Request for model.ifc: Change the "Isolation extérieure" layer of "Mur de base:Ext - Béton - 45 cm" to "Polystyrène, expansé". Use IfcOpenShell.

First a look at what the model holds.

```python
import ifcopenshell
import ifcopenshell.util.element

model = ifcopenshell.open("model.ifc")
print(model.schema)
for layer_set in model.by_type("IfcMaterialLayerSet"):
    if layer_set.LayerSetName == "Mur de base:Ext - Béton - 45 cm":
        for layer in layer_set.MaterialLayers:
            print(layer.id(), layer.Material and layer.Material.Name, layer.LayerThickness, sep=" | ")
        print(len(ifcopenshell.util.element.get_elements_by_material(model, layer_set)), "elements and types use it")
print(sorted(m.Name for m in model.by_type("IfcMaterial") if m.Name)[:60])
```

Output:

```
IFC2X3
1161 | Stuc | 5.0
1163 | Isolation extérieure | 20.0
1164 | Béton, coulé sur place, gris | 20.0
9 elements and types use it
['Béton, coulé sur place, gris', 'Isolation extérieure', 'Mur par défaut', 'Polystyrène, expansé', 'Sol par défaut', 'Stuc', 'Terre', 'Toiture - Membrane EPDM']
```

```python
import ifcopenshell
import ifcopenshell.api.material

model = ifcopenshell.open("model.ifc")

layer_set = next(s for s in model.by_type("IfcMaterialLayerSet") if s.LayerSetName == "Mur de base:Ext - Béton - 45 cm")
layer = next(l for l in layer_set.MaterialLayers if l.Material and l.Material.Name == "Isolation extérieure")
material = next(m for m in model.by_type("IfcMaterial") if m.Name == "Polystyrène, expansé")

# Point this one layer at the other material; renaming the old one would change it everywhere.
ifcopenshell.api.material.edit_layer(model, layer=layer, attributes={}, material=material)

print([l.Material.Name if l.Material else None for l in layer_set.MaterialLayers])

model.write("model_edited.ifc")
```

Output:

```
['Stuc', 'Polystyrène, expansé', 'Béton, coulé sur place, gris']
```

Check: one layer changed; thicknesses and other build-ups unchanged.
